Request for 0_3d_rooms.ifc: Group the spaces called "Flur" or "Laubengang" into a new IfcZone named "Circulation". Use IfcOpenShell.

First a look at what the model holds.

```python
import ifcopenshell

model = ifcopenshell.open("0_3d_rooms.ifc")
print(model.schema)
seen = {}
for space in model.by_type("IfcSpace"):
    seen[space.LongName] = seen.get(space.LongName, 0) + 1
for name, count in sorted(seen.items(), key=str):
    print(count, "x", name)
print("zones:", [z.Name for z in model.by_type("IfcZone")][:20])
```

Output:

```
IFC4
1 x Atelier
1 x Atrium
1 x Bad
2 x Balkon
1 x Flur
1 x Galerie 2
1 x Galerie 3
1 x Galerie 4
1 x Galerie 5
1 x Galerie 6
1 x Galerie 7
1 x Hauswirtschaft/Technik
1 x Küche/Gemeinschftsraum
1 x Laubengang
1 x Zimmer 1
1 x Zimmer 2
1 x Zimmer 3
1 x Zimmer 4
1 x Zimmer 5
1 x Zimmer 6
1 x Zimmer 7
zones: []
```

```python
import ifcopenshell
import ifcopenshell.api.group
import ifcopenshell.api.root

model = ifcopenshell.open("0_3d_rooms.ifc")

names = {"Flur", "Laubengang"}
spaces = [s for s in model.by_type("IfcSpace") if s.LongName in names]

zone = ifcopenshell.api.root.create_entity(model, ifc_class="IfcZone", name="Circulation")
ifcopenshell.api.group.assign_group(model, products=spaces, group=zone)
print(len(spaces), "spaces in", zone.Name)

model.write("0_3d_rooms_rev.ifc")
```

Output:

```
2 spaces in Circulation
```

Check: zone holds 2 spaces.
